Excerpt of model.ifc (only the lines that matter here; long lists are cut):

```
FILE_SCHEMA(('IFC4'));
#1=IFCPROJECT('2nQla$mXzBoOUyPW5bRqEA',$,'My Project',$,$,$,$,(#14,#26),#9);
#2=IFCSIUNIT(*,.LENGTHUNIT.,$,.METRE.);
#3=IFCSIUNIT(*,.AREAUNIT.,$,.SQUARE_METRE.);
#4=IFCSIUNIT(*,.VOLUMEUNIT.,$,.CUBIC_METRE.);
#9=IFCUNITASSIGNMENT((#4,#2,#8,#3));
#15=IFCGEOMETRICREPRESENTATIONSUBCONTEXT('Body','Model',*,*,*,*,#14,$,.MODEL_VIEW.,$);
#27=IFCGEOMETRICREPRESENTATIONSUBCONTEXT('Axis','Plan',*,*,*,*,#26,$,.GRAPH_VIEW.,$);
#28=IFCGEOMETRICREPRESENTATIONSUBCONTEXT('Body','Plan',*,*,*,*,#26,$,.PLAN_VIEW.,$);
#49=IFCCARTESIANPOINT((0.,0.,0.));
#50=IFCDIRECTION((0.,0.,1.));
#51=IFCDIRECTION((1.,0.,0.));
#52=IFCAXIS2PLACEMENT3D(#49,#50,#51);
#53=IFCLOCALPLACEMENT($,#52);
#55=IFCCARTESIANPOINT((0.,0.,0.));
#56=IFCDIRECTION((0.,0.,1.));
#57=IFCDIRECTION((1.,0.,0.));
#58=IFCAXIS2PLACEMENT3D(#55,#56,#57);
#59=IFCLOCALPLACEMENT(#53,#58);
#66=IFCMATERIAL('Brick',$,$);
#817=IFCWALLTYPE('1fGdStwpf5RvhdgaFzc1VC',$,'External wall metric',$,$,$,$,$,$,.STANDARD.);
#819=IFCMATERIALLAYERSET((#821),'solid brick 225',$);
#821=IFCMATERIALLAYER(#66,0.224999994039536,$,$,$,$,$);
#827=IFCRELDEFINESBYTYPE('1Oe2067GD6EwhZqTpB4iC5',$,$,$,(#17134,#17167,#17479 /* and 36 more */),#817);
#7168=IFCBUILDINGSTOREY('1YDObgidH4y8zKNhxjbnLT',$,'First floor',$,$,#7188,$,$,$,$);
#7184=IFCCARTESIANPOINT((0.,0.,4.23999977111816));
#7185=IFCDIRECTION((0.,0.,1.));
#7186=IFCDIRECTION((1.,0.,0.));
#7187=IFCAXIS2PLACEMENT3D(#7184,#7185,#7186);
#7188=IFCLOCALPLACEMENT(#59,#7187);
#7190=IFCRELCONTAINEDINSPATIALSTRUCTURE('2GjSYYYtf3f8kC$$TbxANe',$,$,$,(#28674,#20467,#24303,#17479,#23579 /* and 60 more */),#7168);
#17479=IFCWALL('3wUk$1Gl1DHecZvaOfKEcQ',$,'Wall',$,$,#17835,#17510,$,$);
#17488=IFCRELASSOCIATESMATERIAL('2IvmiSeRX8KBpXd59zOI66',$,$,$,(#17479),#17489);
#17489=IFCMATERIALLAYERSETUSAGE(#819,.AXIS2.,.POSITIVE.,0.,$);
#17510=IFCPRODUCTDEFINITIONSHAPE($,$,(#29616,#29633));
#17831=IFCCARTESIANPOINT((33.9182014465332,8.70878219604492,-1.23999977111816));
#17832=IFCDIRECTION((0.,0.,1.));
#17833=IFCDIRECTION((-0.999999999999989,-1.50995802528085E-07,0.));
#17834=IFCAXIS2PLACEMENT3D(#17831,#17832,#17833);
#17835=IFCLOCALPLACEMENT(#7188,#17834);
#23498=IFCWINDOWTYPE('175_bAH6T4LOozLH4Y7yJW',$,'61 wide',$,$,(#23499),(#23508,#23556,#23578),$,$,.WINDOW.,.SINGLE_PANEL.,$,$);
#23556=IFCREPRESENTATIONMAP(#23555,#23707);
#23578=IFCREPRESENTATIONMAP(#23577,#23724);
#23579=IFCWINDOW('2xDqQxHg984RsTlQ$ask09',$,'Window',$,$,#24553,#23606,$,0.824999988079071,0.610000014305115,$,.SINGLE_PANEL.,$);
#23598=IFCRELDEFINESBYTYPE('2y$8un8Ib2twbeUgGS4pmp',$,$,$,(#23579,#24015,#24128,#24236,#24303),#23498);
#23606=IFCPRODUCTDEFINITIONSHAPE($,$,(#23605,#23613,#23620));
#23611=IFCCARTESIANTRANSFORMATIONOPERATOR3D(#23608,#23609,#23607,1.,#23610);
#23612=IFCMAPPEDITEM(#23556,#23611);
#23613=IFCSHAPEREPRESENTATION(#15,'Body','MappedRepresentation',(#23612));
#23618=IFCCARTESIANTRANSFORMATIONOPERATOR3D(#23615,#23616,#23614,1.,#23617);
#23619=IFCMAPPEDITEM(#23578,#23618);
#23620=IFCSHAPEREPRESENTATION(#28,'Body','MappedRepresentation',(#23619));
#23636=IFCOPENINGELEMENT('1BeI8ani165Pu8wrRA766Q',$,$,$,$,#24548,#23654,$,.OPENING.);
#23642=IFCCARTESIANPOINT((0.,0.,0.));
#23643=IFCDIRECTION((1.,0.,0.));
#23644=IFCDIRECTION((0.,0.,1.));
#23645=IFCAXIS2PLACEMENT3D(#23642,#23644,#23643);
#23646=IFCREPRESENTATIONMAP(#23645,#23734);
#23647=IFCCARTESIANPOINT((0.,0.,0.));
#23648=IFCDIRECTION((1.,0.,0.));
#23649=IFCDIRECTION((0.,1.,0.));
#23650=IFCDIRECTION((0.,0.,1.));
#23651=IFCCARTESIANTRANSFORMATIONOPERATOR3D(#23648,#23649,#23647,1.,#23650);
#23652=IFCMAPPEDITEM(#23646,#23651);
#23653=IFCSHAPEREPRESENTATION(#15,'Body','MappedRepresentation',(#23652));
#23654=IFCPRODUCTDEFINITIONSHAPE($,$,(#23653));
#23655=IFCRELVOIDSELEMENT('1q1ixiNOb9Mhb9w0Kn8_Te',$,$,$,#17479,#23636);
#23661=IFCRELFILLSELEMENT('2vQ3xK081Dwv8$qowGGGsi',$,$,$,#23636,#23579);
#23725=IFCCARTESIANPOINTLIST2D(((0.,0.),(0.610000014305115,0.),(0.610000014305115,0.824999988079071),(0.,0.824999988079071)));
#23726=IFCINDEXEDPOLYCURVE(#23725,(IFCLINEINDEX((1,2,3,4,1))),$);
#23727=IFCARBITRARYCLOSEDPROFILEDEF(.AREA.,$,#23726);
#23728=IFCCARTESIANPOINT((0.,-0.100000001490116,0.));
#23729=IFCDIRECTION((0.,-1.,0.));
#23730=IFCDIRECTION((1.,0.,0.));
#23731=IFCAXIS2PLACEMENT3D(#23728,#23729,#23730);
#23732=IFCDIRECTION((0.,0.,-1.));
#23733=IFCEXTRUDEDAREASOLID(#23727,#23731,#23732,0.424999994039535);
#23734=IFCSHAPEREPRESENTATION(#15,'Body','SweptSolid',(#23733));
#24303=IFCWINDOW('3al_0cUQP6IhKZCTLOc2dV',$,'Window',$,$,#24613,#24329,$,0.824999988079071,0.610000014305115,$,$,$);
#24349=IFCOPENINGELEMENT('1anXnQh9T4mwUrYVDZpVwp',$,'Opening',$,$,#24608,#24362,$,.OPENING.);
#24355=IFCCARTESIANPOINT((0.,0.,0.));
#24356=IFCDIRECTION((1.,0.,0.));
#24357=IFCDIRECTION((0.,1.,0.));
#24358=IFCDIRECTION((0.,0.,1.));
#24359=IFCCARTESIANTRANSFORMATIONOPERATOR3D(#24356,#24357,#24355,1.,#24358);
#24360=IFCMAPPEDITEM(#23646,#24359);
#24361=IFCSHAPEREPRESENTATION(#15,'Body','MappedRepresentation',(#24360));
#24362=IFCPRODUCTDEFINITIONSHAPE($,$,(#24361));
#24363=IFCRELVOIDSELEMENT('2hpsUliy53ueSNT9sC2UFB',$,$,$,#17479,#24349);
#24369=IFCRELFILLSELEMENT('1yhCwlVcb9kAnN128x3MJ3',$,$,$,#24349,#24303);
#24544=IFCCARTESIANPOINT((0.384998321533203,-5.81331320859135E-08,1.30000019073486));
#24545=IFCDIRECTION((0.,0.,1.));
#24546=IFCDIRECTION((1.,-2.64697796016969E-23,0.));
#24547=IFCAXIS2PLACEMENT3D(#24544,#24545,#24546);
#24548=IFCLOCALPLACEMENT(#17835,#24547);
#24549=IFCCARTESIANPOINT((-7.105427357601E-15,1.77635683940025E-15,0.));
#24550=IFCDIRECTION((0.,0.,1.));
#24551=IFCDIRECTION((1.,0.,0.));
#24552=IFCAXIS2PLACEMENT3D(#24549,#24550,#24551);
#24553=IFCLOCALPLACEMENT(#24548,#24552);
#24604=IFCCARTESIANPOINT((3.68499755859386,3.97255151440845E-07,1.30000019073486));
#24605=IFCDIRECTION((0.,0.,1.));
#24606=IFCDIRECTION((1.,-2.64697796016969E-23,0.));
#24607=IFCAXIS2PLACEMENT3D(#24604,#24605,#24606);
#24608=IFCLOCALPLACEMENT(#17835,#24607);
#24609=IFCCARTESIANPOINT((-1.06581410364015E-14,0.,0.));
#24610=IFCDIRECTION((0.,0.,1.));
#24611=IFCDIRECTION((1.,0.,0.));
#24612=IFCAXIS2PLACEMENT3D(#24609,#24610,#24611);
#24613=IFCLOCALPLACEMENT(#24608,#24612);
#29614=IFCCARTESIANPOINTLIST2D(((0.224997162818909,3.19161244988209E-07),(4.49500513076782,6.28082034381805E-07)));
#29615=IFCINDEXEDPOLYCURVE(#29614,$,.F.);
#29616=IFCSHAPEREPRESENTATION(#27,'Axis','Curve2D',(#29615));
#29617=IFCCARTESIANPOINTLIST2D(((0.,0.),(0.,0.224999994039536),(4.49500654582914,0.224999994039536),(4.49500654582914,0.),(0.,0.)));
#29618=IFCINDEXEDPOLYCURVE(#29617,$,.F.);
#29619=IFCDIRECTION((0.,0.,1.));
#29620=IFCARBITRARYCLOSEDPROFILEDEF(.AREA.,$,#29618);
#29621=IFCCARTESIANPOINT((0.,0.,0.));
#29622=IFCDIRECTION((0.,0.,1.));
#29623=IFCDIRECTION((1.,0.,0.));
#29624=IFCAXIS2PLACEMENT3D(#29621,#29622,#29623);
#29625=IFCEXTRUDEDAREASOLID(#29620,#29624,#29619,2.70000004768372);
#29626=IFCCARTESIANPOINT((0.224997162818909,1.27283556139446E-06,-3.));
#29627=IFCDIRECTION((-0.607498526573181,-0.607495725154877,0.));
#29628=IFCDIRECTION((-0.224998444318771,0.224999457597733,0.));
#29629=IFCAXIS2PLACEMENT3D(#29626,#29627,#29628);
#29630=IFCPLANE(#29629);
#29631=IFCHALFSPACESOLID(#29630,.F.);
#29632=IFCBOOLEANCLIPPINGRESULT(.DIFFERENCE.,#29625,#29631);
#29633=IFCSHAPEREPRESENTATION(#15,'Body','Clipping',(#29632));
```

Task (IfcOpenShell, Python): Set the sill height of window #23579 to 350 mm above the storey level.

```python
import numpy as np
import ifcopenshell
import ifcopenshell.api.geometry
import ifcopenshell.geom
import ifcopenshell.util.element
import ifcopenshell.util.placement
import ifcopenshell.util.shape
import ifcopenshell.util.unit

model = ifcopenshell.open("model.ifc")
unit_scale = ifcopenshell.util.unit.calculate_unit_scale(model)

window = model.by_guid("2xDqQxHg984RsTlQ$ask09")
opening = window.FillsVoids[0].RelatingOpeningElement
storey = ifcopenshell.util.element.get_container(window, ifc_class="IfcBuildingStorey")
level = ifcopenshell.util.placement.get_local_placement(storey.ObjectPlacement)[2, 3]

# The opening's origin need not be at the sill, so measure its lowest point.
shape = ifcopenshell.geom.create_shape(ifcopenshell.geom.settings(), opening)
bottom = ifcopenshell.util.shape.get_shape_bottom_elevation(shape, shape.geometry) / unit_scale
dz = level + 0.35 / unit_scale - bottom

shift = np.array([0.0, 0.0, dz])
# The window is placed relative to its opening, so it follows when the opening moves.
matrix = ifcopenshell.util.placement.get_local_placement(opening.ObjectPlacement)
matrix[:3, 3] += shift
ifcopenshell.api.geometry.edit_object_placement(
    model, product=opening, matrix=matrix, is_si=False, should_transform_children=True
)

print(f"moved by {dz * unit_scale:+.3f} m")

model.write("model-out.ifc")
```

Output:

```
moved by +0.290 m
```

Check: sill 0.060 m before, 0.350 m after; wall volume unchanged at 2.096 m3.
